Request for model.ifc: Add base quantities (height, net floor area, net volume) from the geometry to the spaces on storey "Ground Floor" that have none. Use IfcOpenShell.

First a look at what the model holds.

```python
import ifcopenshell
import ifcopenshell.util.element
import ifcopenshell.util.unit

model = ifcopenshell.open("model.ifc")
print(model.schema)
for unit_type in ("LENGTHUNIT", "AREAUNIT", "VOLUMEUNIT"):
    print(unit_type, ifcopenshell.util.unit.calculate_unit_scale(model, unit_type))
storey = next(s for s in model.by_type("IfcBuildingStorey") if s.Name == "Ground Floor")
spaces = [e for e in ifcopenshell.util.element.get_decomposition(storey) if e.is_a("IfcSpace")]
for e in sorted(spaces, key=lambda e: e.id()):
    print(e.id(), e.is_a(), e.Name, list(ifcopenshell.util.element.get_psets(e, qtos_only=True)), sep=" | ")
```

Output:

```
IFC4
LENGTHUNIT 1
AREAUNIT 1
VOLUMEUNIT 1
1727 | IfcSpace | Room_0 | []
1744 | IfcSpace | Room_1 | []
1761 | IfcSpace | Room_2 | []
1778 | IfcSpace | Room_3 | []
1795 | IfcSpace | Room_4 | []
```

```python
import ifcopenshell
import ifcopenshell.api.pset
import ifcopenshell.geom
import ifcopenshell.util.element
import ifcopenshell.util.shape
import ifcopenshell.util.unit

model = ifcopenshell.open("model.ifc")
unit_scale = ifcopenshell.util.unit.calculate_unit_scale(model)
area_scale = ifcopenshell.util.unit.calculate_unit_scale(model, "AREAUNIT")
volume_scale = ifcopenshell.util.unit.calculate_unit_scale(model, "VOLUMEUNIT")
settings = ifcopenshell.geom.settings()

storey = next(s for s in model.by_type("IfcBuildingStorey") if s.Name == "Ground Floor")
spaces = [e for e in ifcopenshell.util.element.get_decomposition(storey) if e.is_a("IfcSpace")]

for e in sorted(spaces, key=lambda e: e.id()):
    if ifcopenshell.util.element.get_psets(e, qtos_only=True, should_inherit=False):
        continue
    # Geometry comes back in metres, in the element's own axes.
    shape = ifcopenshell.geom.create_shape(settings, e)
    values = {
        "Height": ifcopenshell.util.shape.get_z(shape.geometry) / unit_scale,
        "NetFloorArea": ifcopenshell.util.shape.get_footprint_area(shape.geometry) / area_scale,
        "NetVolume": ifcopenshell.util.shape.get_volume(shape.geometry) / volume_scale,
    }
    qto = ifcopenshell.api.pset.add_qto(model, product=e, name="Qto_SpaceBaseQuantities")
    ifcopenshell.api.pset.edit_qto(model, qto=qto, properties=values)
    print(e.id(), {k: round(v, 3) for k, v in values.items()})

model.write("model_updated.ifc")
```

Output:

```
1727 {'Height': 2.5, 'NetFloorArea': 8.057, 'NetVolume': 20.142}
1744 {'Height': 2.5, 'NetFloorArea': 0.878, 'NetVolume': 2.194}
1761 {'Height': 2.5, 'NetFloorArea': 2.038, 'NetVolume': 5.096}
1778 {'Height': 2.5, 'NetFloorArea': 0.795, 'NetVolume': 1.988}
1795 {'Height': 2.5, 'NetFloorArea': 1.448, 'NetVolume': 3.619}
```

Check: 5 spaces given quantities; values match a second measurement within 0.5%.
